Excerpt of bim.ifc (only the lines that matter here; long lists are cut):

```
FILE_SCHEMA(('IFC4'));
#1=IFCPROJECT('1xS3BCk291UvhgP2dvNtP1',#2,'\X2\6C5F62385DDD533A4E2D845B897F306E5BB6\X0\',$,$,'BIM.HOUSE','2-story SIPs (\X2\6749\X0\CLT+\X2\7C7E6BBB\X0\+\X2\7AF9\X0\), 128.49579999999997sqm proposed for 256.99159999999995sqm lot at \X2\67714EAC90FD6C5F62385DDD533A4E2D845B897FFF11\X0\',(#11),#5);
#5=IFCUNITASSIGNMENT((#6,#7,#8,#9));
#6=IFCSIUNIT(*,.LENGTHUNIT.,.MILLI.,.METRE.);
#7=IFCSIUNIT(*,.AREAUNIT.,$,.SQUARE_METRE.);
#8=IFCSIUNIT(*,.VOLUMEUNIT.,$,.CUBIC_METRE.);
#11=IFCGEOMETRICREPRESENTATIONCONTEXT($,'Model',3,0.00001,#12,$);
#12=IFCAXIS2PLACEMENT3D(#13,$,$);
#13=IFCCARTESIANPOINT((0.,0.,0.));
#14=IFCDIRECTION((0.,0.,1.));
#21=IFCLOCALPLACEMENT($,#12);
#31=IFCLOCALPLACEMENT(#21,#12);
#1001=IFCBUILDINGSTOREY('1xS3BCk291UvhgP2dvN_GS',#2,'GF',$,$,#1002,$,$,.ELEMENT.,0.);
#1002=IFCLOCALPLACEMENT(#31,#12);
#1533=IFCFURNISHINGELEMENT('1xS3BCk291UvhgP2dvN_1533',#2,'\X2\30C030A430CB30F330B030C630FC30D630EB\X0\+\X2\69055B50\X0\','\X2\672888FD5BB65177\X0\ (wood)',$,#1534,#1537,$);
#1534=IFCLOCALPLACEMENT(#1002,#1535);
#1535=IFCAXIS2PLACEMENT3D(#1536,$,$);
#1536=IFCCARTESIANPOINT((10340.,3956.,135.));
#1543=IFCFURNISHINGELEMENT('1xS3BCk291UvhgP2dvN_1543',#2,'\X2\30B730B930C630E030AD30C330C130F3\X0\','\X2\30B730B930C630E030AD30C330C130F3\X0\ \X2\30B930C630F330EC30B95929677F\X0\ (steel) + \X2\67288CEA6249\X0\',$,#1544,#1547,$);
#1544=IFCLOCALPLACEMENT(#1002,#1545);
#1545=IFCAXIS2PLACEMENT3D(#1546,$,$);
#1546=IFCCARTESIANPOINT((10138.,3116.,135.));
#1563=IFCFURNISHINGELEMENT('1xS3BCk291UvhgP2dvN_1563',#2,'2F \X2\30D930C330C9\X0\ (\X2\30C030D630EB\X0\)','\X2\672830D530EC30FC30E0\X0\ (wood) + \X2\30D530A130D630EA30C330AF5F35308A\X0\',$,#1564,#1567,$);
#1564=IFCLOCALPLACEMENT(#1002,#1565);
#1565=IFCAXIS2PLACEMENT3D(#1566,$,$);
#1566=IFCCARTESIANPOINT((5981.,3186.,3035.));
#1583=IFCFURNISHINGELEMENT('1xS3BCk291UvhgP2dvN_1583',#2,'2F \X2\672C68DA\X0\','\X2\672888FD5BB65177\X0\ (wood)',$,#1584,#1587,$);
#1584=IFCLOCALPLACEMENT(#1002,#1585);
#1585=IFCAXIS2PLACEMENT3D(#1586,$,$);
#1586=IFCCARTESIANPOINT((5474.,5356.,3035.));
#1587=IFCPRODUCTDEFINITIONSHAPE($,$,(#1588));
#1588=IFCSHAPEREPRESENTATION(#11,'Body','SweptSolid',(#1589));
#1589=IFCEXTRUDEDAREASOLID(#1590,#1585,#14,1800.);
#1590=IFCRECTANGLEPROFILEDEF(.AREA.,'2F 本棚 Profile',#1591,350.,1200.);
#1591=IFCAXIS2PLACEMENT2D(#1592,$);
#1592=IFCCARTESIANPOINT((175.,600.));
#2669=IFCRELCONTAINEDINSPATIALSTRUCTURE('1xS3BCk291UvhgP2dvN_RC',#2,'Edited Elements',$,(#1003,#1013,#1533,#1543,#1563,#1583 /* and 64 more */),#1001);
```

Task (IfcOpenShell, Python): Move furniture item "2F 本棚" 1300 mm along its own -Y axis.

```python
import ifcopenshell
import ifcopenshell.api.geometry
import ifcopenshell.util.placement

model = ifcopenshell.open("bim.ifc")

item = model.by_guid("1xS3BCk291UvhgP2dvN_1583")
matrix = ifcopenshell.util.placement.get_local_placement(item.ObjectPlacement)
matrix[:3, 3] -= matrix[:3, 1] * 1300.0
ifcopenshell.api.geometry.edit_object_placement(model, product=item, matrix=matrix, is_si=False)

print(ifcopenshell.util.placement.get_local_placement(item.ObjectPlacement).round(3) + 0.0)

model.write("bim_edited.ifc")
```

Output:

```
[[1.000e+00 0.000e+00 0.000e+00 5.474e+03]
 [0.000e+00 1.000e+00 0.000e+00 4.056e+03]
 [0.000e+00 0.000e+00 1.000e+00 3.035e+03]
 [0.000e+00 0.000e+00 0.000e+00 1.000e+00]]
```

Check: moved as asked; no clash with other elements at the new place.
